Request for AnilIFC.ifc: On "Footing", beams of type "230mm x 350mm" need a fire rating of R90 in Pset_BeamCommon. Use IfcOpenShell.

First a look at what the model holds.

```python
import ifcopenshell
import ifcopenshell.util.element

model = ifcopenshell.open("AnilIFC.ifc")
print(model.schema)
storey = next(s for s in model.by_type("IfcBuildingStorey") if s.Name == "Footing")
beams = [e for e in ifcopenshell.util.element.get_decomposition(storey) if e.is_a("IfcBeam")]
seen = {}
for e in beams:
    element_type = ifcopenshell.util.element.get_type(e)
    key = (element_type.Name if element_type != e and element_type else None, ifcopenshell.util.element.get_pset(e, "Pset_BeamCommon", "FireRating"))
    seen[key] = seen.get(key, 0) + 1
for (name, value), count in sorted(seen.items(), key=str):
    print(count, "x", name, "|", value)
```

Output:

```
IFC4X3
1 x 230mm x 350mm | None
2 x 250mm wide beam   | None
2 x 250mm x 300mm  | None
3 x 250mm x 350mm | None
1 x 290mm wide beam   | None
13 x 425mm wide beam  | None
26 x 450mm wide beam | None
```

```python
import ifcopenshell
import ifcopenshell.api.pset
import ifcopenshell.util.element

model = ifcopenshell.open("AnilIFC.ifc")

storey = next(s for s in model.by_type("IfcBuildingStorey") if s.Name == "Footing")
beams = [e for e in ifcopenshell.util.element.get_decomposition(storey) if e.is_a("IfcBeam")]

count = 0
for e in beams:
    element_type = ifcopenshell.util.element.get_type(e)
    if element_type in (None, e) or element_type.Name != "230mm x 350mm":
        continue
    # add_pset returns the element's existing set when there is one.
    pset = ifcopenshell.api.pset.add_pset(model, product=e, name="Pset_BeamCommon")
    ifcopenshell.api.pset.edit_pset(model, pset=pset, properties={"FireRating": "R90"})
    count += 1

print(count, "beams updated")

model.write("AnilIFC_updated.ifc")
```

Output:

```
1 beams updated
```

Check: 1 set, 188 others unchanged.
